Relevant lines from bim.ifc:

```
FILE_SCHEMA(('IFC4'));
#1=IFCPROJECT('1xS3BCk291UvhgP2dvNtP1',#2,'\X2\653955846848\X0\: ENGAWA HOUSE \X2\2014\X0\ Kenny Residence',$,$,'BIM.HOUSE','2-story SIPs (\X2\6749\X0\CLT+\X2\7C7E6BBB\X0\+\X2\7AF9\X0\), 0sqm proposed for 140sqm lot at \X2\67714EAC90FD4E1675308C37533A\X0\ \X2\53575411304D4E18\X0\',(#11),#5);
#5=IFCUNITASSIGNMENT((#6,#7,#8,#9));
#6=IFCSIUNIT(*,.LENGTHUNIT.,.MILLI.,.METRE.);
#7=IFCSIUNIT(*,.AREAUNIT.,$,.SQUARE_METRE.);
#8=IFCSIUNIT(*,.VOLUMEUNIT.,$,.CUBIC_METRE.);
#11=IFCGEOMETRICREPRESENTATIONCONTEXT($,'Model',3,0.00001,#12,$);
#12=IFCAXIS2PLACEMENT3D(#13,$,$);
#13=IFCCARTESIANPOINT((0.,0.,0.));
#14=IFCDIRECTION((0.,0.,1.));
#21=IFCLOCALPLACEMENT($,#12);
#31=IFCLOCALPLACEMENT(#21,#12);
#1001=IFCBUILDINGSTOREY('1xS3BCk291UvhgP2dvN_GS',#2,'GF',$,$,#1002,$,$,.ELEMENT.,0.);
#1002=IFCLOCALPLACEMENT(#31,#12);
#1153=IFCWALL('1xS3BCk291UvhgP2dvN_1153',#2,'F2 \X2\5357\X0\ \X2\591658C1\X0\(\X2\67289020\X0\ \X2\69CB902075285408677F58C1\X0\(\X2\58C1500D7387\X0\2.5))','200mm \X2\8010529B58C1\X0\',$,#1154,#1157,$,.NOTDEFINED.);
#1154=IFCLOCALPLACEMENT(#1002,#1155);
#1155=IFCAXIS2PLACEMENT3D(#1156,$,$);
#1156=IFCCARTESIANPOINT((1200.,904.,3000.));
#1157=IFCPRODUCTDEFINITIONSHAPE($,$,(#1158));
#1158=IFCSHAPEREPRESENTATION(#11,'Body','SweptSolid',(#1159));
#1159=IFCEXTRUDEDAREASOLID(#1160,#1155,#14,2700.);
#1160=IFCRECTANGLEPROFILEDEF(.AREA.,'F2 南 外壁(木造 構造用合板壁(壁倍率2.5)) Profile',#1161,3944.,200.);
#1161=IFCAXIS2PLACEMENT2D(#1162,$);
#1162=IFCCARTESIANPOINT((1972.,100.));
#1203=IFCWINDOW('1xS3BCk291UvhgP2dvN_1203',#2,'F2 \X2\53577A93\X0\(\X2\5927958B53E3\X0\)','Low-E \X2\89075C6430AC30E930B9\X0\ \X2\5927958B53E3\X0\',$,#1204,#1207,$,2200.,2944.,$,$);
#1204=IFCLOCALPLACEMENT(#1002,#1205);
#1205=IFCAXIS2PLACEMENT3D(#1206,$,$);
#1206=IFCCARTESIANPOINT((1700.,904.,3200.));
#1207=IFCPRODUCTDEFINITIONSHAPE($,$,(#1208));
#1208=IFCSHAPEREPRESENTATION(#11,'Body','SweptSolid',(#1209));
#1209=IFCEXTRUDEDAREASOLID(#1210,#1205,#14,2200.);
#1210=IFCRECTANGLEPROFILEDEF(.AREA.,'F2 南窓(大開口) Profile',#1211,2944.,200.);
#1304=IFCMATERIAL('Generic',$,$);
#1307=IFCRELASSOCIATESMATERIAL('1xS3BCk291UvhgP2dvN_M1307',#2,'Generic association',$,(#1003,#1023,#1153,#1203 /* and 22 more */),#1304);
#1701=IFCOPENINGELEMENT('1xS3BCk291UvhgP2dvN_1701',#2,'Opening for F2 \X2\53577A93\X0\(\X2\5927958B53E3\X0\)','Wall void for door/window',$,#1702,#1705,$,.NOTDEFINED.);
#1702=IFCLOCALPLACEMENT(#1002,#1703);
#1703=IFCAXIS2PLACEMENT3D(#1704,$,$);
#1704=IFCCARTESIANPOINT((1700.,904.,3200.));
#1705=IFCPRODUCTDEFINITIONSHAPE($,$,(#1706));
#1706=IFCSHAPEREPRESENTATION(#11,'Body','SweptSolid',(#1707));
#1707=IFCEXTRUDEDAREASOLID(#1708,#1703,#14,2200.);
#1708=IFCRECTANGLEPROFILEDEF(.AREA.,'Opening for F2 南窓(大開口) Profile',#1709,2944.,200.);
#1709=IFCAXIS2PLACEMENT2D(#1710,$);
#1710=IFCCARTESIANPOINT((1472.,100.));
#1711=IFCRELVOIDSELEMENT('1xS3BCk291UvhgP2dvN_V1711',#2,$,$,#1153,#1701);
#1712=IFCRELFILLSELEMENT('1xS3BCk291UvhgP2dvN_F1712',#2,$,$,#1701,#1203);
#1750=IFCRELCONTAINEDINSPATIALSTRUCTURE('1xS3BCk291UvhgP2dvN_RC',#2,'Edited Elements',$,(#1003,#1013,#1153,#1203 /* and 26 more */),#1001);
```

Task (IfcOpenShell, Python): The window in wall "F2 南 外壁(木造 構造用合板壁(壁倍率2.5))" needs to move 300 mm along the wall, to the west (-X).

```python
import ifcopenshell
import ifcopenshell.api.geometry
import ifcopenshell.util.placement

model = ifcopenshell.open("bim.ifc")

window = model.by_guid("1xS3BCk291UvhgP2dvN_1203")
opening = window.FillsVoids[0].RelatingOpeningElement
wall = opening.VoidsElements[0].RelatingBuildingElement

wall_matrix = ifcopenshell.util.placement.get_local_placement(wall.ObjectPlacement)
shift = wall_matrix[:3, 0] * -300.0
before = ifcopenshell.util.placement.get_local_placement(window.ObjectPlacement)[:3, 3].copy()

# The window is not placed relative to its opening, so move both.
for product in (opening, window):
    matrix = ifcopenshell.util.placement.get_local_placement(product.ObjectPlacement)
    matrix[:3, 3] += shift
    ifcopenshell.api.geometry.edit_object_placement(model, product=product, matrix=matrix, is_si=False)

after = ifcopenshell.util.placement.get_local_placement(window.ObjectPlacement)[:3, 3]
print("window moved by", (after - before).round(3) + 0.0)

model.write("bim-out.ifc")
```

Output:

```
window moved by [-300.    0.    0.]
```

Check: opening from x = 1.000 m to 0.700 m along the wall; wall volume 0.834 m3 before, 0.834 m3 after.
